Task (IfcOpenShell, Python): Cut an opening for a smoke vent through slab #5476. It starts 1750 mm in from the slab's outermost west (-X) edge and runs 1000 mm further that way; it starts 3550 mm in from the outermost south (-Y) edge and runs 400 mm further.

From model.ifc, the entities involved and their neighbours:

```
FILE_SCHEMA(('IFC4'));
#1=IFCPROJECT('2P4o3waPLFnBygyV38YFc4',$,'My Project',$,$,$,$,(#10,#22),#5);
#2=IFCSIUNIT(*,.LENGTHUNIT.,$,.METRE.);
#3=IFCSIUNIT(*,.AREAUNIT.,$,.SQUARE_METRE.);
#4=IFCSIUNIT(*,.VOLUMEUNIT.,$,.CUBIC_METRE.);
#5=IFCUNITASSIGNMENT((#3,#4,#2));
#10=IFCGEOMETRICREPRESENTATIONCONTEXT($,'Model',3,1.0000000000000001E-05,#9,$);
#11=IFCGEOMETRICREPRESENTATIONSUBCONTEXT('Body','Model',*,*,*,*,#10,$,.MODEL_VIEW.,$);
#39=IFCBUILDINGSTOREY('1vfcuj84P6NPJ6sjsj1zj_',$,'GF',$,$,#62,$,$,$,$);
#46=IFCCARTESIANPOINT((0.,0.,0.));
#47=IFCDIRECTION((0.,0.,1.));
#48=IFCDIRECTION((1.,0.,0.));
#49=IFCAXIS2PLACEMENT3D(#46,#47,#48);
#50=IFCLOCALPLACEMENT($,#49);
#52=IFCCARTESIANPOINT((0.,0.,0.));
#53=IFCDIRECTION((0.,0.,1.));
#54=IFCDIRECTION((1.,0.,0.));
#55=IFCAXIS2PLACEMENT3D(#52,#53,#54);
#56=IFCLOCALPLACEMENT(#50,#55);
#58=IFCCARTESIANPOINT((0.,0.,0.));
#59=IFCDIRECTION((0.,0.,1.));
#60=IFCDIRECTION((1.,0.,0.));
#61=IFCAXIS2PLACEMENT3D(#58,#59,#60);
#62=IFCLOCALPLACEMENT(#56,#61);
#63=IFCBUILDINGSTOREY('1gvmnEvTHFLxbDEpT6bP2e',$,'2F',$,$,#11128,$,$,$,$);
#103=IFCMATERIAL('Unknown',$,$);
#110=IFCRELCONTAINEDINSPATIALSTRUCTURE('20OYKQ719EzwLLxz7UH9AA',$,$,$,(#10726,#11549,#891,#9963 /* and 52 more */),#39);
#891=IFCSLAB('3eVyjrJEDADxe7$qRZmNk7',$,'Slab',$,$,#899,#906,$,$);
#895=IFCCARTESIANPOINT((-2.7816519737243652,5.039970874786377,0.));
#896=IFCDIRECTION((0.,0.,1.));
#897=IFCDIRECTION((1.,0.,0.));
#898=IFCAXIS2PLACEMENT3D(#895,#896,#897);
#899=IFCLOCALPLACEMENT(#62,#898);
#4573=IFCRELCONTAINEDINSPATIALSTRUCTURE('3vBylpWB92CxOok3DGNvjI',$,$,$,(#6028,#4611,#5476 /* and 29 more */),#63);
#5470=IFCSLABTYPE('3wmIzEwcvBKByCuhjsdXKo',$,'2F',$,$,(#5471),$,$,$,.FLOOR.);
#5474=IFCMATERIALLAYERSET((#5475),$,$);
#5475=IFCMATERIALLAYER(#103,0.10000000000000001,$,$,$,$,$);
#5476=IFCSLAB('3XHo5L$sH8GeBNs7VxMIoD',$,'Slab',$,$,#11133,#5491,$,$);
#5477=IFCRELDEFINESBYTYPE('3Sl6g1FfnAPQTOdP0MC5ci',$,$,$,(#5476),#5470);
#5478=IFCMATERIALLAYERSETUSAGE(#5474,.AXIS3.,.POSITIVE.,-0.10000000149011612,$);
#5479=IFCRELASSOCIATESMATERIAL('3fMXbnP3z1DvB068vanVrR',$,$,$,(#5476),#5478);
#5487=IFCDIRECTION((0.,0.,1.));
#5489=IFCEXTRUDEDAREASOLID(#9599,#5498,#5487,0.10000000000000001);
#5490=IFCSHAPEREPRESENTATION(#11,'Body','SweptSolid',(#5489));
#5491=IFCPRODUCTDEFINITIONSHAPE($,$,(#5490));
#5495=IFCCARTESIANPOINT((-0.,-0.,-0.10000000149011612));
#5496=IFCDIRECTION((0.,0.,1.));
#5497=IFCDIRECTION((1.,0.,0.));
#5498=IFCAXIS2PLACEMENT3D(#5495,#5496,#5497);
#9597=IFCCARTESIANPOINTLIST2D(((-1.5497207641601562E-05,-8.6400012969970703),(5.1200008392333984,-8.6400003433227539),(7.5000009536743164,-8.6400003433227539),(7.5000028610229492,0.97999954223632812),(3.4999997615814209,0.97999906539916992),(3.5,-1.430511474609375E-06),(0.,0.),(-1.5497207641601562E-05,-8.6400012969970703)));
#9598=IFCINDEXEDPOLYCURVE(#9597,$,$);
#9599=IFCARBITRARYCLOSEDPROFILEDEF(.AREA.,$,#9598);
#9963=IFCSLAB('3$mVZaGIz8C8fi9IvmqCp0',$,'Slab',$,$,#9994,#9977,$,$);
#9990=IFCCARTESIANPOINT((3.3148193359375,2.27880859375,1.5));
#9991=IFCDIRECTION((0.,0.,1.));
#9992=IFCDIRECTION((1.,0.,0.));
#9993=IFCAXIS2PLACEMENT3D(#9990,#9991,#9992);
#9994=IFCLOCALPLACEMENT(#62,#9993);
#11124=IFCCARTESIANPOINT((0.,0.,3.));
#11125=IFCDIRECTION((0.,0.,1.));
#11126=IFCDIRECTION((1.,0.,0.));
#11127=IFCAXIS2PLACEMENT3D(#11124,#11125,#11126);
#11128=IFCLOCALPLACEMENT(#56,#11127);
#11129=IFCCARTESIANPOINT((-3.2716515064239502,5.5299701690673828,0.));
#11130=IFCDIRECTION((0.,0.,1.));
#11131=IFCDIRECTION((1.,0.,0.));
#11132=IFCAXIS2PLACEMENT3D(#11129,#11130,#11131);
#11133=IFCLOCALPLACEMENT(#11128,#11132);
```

```python
import numpy as np
import ifcopenshell
import ifcopenshell.api.feature
import ifcopenshell.api.geometry
import ifcopenshell.api.root
import ifcopenshell.geom
import ifcopenshell.util.placement
import ifcopenshell.util.representation
import ifcopenshell.util.shape
import ifcopenshell.util.unit

model = ifcopenshell.open("model.ifc")
unit_scale = ifcopenshell.util.unit.calculate_unit_scale(model)
settings = ifcopenshell.geom.settings()


def volume(element):
    """Net volume in cubic metres, openings subtracted."""
    shape = ifcopenshell.geom.create_shape(settings, element)
    return ifcopenshell.util.shape.get_volume(shape.geometry)


slab = model.by_guid("3XHo5L$sH8GeBNs7VxMIoD")
before = volume(slab)

# Extent in the slab's own axes, in metres. The edges named are its -X and -Y sides.
slab_shape = ifcopenshell.geom.create_shape(settings, slab)
vertices = ifcopenshell.util.shape.get_vertices(slab_shape.geometry)
x_min, y_min, bottom = vertices.min(axis=0)
top = vertices[:, 2].max()

opening = ifcopenshell.api.root.create_entity(model, ifc_class="IfcOpeningElement", name="Smoke vent opening", predefined_type="OPENING")
context = ifcopenshell.util.representation.get_context(model, "Model", "Body", "MODEL_VIEW")
width, depth = 1, 0.4
outline = [(0.0, 0.0), (width, 0.0), (width, depth), (0.0, depth), (0.0, 0.0)]
# Overshoot both faces by 50 mm so the cut is clean.
shape = ifcopenshell.api.geometry.add_slab_representation(
    model, context=context, depth=top - bottom + 0.1, polyline=outline
)
ifcopenshell.api.geometry.assign_representation(model, product=opening, representation=shape)

matrix = ifcopenshell.util.placement.get_local_placement(slab.ObjectPlacement)
matrix[:, 3] = matrix @ np.append(np.array([x_min + 1.75, y_min + 3.55, bottom - 0.05]) / unit_scale, 1.0)
ifcopenshell.api.geometry.edit_object_placement(model, product=opening, matrix=matrix, is_si=False)
ifcopenshell.api.feature.add_feature(model, feature=opening, element=slab)

after = volume(slab)

print(f"slab volume {before:.3f} -> {after:.3f} m3")

model.write("model_edited.ifc")
```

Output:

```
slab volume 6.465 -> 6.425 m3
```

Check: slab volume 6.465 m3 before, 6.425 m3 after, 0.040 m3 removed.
